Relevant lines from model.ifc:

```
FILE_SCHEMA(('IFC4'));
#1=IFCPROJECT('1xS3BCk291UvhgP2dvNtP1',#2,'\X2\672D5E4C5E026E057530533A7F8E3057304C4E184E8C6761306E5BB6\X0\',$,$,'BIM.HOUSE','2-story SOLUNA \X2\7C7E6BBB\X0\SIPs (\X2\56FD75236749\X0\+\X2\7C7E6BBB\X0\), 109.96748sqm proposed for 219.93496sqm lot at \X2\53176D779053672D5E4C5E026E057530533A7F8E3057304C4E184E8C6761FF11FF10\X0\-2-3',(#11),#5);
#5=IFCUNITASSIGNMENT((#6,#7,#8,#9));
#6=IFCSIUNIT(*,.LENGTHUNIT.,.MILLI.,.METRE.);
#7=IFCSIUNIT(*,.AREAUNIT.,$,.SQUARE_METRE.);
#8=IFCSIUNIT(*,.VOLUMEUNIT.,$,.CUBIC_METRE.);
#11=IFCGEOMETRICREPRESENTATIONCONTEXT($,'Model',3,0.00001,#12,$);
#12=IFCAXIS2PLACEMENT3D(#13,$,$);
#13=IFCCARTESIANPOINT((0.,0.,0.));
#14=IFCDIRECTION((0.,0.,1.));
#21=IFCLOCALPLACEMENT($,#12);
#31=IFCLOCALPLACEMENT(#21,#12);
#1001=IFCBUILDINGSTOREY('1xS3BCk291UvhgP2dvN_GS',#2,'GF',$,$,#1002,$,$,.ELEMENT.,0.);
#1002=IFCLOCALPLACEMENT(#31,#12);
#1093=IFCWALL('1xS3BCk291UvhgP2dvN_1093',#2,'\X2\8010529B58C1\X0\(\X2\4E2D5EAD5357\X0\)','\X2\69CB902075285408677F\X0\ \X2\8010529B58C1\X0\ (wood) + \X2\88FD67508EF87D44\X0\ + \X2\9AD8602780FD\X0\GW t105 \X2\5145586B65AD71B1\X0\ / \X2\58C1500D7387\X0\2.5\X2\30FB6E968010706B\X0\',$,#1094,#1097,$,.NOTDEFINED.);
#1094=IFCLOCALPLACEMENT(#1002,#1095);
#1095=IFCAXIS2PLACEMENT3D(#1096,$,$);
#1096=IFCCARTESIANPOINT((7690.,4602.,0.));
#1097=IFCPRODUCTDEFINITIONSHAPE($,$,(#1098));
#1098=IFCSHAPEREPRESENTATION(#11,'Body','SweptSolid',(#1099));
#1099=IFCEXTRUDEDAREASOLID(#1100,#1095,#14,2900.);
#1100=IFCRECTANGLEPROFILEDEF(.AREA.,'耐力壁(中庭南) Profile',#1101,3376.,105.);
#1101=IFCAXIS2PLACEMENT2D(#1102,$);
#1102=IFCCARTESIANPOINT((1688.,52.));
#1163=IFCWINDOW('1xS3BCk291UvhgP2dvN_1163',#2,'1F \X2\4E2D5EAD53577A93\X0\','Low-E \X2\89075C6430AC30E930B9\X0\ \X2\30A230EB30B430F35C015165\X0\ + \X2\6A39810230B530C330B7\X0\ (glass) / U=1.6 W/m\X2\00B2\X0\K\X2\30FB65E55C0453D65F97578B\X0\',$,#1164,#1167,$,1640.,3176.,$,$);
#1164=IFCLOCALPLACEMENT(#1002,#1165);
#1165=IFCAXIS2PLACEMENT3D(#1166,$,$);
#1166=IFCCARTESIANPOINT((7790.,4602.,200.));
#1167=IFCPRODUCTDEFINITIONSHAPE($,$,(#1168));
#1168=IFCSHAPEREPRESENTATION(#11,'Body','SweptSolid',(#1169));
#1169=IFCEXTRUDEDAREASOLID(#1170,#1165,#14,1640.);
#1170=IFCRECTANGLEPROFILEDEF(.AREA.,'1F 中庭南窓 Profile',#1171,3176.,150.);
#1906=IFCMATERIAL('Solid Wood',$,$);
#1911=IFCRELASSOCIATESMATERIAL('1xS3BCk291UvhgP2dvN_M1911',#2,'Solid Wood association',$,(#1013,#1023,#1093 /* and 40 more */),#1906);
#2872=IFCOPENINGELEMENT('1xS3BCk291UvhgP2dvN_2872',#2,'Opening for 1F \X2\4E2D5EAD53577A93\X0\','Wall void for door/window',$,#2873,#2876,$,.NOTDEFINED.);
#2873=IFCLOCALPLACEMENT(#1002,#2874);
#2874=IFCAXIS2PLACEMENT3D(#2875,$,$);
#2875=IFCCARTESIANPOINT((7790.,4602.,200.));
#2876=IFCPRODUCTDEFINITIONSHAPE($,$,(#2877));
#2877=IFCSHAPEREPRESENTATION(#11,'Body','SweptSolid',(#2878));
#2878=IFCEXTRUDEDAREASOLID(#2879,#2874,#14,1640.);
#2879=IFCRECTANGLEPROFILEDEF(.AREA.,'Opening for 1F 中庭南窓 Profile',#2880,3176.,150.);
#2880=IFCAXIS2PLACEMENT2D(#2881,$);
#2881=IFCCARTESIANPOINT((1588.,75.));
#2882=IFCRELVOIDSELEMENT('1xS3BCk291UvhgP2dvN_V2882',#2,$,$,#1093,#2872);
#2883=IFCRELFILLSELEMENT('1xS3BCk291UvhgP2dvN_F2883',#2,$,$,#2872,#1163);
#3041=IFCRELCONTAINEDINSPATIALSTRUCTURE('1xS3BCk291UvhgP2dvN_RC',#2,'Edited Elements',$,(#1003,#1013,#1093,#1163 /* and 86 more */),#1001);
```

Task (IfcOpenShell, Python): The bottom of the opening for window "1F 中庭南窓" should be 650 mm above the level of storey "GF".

```python
import numpy as np
import ifcopenshell
import ifcopenshell.api.geometry
import ifcopenshell.geom
import ifcopenshell.util.element
import ifcopenshell.util.placement
import ifcopenshell.util.shape
import ifcopenshell.util.unit

model = ifcopenshell.open("model.ifc")
unit_scale = ifcopenshell.util.unit.calculate_unit_scale(model)

window = model.by_guid("1xS3BCk291UvhgP2dvN_1163")
opening = window.FillsVoids[0].RelatingOpeningElement
storey = ifcopenshell.util.element.get_container(window, ifc_class="IfcBuildingStorey")
level = ifcopenshell.util.placement.get_local_placement(storey.ObjectPlacement)[2, 3]

# The opening's origin need not be at the sill, so measure its lowest point.
shape = ifcopenshell.geom.create_shape(ifcopenshell.geom.settings(), opening)
bottom = ifcopenshell.util.shape.get_shape_bottom_elevation(shape, shape.geometry) / unit_scale
dz = level + 0.65 / unit_scale - bottom

shift = np.array([0.0, 0.0, dz])
# The window is not placed relative to its opening, so move both.
for product in (opening, window):
    matrix = ifcopenshell.util.placement.get_local_placement(product.ObjectPlacement)
    matrix[:3, 3] += shift
    ifcopenshell.api.geometry.edit_object_placement(model, product=product, matrix=matrix, is_si=False)

print(f"moved by {dz * unit_scale:+.3f} m")

model.write("model_v2.ifc")
```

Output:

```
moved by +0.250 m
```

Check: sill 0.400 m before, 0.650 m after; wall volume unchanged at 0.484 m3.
